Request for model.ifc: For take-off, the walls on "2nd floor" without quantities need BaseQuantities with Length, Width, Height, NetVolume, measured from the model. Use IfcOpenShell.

First a look at what the model holds.

```python
import ifcopenshell
import ifcopenshell.util.element
import ifcopenshell.util.unit

model = ifcopenshell.open("model.ifc")
print(model.schema)
for unit_type in ("LENGTHUNIT", "AREAUNIT", "VOLUMEUNIT"):
    print(unit_type, ifcopenshell.util.unit.calculate_unit_scale(model, unit_type))
storey = next(s for s in model.by_type("IfcBuildingStorey") if s.Name == "2nd floor")
walls = [e for e in ifcopenshell.util.element.get_decomposition(storey) if e.is_a("IfcWall")]
for e in sorted(walls, key=lambda e: e.id()):
    print(e.id(), e.is_a(), e.Name, list(ifcopenshell.util.element.get_psets(e, qtos_only=True)), sep=" | ")
```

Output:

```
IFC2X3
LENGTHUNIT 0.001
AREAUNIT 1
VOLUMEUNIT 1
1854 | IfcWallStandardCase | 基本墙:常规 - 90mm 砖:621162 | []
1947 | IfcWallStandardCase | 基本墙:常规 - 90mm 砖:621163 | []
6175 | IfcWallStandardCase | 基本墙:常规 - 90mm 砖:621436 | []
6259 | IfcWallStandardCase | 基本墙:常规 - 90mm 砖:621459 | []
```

```python
import ifcopenshell
import ifcopenshell.api.pset
import ifcopenshell.geom
import ifcopenshell.util.element
import ifcopenshell.util.shape
import ifcopenshell.util.unit

model = ifcopenshell.open("model.ifc")
unit_scale = ifcopenshell.util.unit.calculate_unit_scale(model)
volume_scale = ifcopenshell.util.unit.calculate_unit_scale(model, "VOLUMEUNIT")
settings = ifcopenshell.geom.settings()

storey = next(s for s in model.by_type("IfcBuildingStorey") if s.Name == "2nd floor")
walls = [e for e in ifcopenshell.util.element.get_decomposition(storey) if e.is_a("IfcWall")]

for e in sorted(walls, key=lambda e: e.id()):
    if ifcopenshell.util.element.get_psets(e, qtos_only=True, should_inherit=False):
        continue
    # Geometry comes back in metres, in the element's own axes.
    shape = ifcopenshell.geom.create_shape(settings, e)
    values = {
        "Length": ifcopenshell.util.shape.get_x(shape.geometry) / unit_scale,
        "Width": ifcopenshell.util.shape.get_y(shape.geometry) / unit_scale,
        "Height": ifcopenshell.util.shape.get_z(shape.geometry) / unit_scale,
        "NetVolume": ifcopenshell.util.shape.get_volume(shape.geometry) / volume_scale,
    }
    qto = ifcopenshell.api.pset.add_qto(model, product=e, name="BaseQuantities")
    ifcopenshell.api.pset.edit_qto(model, qto=qto, properties=values)
    print(e.id(), {k: round(v, 3) for k, v in values.items()})

model.write("model_rev.ifc")
```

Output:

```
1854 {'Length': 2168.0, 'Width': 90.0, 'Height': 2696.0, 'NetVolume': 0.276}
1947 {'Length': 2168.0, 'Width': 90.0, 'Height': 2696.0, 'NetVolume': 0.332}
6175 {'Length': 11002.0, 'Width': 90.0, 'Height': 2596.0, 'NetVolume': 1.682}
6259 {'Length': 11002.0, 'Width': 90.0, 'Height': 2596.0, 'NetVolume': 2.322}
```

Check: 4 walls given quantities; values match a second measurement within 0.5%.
